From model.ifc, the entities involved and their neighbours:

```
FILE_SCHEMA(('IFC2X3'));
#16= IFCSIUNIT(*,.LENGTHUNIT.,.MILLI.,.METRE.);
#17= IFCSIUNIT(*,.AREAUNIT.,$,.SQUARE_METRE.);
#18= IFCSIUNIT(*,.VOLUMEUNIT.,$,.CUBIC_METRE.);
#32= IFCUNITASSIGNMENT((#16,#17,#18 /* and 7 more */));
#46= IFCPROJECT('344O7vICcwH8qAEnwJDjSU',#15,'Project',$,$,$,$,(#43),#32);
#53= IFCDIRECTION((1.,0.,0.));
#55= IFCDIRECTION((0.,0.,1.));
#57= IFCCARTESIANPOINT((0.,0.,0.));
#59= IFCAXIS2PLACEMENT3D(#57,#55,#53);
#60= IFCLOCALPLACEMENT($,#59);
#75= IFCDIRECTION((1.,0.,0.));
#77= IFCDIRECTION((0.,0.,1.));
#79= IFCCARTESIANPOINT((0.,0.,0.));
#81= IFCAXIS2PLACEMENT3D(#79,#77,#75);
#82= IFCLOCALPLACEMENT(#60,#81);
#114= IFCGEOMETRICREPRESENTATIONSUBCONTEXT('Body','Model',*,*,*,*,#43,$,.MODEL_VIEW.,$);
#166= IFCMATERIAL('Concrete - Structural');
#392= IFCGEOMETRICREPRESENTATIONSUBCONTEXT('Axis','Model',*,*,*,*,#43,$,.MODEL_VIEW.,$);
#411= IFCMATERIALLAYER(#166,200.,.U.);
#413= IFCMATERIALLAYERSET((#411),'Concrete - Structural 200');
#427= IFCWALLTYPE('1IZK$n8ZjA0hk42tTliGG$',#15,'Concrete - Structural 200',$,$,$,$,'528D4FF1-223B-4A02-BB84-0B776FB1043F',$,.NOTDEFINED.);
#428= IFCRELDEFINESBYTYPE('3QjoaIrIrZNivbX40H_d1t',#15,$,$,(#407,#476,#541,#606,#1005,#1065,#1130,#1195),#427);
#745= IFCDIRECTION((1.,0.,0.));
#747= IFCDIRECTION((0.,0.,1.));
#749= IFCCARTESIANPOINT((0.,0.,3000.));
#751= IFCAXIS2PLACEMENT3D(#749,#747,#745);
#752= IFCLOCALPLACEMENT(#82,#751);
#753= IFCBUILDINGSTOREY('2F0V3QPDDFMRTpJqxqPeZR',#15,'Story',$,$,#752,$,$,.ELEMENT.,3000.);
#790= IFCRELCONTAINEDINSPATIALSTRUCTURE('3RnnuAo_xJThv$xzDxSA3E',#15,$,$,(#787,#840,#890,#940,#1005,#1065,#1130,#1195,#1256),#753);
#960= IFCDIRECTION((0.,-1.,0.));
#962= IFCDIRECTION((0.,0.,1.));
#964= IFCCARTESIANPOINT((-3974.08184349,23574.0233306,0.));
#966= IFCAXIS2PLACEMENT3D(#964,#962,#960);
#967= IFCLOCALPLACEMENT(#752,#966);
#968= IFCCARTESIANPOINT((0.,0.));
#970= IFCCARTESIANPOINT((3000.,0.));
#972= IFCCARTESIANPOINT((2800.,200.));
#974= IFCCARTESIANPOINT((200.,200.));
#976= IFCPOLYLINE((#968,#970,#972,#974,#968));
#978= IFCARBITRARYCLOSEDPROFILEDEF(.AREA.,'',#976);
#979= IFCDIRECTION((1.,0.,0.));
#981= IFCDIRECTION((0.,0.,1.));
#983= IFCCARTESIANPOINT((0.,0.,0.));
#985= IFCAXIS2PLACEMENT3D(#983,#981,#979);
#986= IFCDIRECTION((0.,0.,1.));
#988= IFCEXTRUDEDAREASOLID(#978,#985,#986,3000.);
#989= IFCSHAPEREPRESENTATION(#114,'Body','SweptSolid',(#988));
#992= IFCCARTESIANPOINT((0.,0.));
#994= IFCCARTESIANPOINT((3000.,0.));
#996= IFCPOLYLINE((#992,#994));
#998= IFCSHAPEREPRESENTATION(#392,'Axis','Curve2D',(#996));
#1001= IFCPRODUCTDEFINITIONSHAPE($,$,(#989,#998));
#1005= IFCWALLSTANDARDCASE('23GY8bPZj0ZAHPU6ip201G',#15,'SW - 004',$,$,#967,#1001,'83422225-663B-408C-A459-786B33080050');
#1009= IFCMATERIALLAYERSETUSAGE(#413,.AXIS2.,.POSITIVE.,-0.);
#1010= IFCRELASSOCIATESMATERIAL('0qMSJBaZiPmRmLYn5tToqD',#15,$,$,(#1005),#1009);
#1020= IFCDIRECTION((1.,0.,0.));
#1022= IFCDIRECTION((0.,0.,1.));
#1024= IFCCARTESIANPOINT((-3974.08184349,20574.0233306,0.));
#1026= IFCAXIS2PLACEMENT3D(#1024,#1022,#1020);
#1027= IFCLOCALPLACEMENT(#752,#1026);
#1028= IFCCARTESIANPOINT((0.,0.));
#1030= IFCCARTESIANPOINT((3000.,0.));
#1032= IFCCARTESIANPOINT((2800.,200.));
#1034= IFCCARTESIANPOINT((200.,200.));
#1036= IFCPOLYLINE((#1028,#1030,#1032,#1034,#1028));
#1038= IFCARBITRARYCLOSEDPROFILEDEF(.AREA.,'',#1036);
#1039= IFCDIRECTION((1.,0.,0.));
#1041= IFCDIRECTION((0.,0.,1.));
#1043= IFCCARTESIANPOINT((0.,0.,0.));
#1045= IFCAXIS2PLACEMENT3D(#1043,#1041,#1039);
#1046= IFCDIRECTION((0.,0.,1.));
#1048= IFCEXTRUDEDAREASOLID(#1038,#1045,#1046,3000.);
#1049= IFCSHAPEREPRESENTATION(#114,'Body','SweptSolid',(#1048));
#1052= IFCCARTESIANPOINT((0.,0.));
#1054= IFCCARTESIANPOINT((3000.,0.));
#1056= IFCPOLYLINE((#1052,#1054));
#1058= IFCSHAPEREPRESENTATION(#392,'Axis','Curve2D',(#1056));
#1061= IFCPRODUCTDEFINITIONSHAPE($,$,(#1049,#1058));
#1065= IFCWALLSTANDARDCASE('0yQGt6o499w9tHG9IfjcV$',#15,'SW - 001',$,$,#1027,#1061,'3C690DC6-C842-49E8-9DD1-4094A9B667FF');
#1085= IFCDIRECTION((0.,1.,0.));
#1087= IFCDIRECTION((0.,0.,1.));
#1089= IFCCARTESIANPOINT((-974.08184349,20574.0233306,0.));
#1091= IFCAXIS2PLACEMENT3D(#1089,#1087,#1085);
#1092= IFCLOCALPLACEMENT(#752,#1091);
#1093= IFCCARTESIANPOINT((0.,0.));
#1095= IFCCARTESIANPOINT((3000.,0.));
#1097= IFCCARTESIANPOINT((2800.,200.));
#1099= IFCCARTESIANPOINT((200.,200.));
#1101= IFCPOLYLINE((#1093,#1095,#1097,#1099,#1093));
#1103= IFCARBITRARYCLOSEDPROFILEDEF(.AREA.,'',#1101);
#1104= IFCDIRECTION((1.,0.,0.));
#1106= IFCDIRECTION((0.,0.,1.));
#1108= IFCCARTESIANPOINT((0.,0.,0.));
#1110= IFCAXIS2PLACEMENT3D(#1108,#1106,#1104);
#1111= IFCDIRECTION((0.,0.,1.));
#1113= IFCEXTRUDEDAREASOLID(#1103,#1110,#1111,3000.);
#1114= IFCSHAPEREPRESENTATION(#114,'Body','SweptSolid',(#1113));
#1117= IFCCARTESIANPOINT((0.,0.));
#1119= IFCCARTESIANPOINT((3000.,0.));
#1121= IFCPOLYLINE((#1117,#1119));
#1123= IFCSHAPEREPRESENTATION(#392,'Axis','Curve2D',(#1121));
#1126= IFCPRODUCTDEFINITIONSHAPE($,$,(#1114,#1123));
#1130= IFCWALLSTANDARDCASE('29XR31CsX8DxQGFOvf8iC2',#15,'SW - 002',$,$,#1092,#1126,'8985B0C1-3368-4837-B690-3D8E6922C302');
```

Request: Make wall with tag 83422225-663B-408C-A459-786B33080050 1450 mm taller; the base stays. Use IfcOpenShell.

```python
import ifcopenshell
import ifcopenshell.geom
import ifcopenshell.util.representation
import ifcopenshell.util.shape
import ifcopenshell.util.unit

model = ifcopenshell.open("model.ifc")
unit_scale = ifcopenshell.util.unit.calculate_unit_scale(model)
settings = ifcopenshell.geom.settings()


def volume(element):
    """Net volume in cubic metres, openings subtracted."""
    shape = ifcopenshell.geom.create_shape(settings, element)
    return ifcopenshell.util.shape.get_volume(shape.geometry)


wall = model.by_guid("23GY8bPZj0ZAHPU6ip201G")
before = volume(wall)

body = ifcopenshell.util.representation.get_representation(wall, "Model", "Body")
solid = body.Items[0]
old_height = solid.Depth
solid.Depth += 1.45 / unit_scale
after = volume(wall)

print(f"height {old_height:g} -> {solid.Depth:g}, volume {before:.3f} -> {after:.3f} m3")

model.write("model_v2.ifc")
```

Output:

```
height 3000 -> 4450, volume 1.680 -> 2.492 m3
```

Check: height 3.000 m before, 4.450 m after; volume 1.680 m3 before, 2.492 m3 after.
